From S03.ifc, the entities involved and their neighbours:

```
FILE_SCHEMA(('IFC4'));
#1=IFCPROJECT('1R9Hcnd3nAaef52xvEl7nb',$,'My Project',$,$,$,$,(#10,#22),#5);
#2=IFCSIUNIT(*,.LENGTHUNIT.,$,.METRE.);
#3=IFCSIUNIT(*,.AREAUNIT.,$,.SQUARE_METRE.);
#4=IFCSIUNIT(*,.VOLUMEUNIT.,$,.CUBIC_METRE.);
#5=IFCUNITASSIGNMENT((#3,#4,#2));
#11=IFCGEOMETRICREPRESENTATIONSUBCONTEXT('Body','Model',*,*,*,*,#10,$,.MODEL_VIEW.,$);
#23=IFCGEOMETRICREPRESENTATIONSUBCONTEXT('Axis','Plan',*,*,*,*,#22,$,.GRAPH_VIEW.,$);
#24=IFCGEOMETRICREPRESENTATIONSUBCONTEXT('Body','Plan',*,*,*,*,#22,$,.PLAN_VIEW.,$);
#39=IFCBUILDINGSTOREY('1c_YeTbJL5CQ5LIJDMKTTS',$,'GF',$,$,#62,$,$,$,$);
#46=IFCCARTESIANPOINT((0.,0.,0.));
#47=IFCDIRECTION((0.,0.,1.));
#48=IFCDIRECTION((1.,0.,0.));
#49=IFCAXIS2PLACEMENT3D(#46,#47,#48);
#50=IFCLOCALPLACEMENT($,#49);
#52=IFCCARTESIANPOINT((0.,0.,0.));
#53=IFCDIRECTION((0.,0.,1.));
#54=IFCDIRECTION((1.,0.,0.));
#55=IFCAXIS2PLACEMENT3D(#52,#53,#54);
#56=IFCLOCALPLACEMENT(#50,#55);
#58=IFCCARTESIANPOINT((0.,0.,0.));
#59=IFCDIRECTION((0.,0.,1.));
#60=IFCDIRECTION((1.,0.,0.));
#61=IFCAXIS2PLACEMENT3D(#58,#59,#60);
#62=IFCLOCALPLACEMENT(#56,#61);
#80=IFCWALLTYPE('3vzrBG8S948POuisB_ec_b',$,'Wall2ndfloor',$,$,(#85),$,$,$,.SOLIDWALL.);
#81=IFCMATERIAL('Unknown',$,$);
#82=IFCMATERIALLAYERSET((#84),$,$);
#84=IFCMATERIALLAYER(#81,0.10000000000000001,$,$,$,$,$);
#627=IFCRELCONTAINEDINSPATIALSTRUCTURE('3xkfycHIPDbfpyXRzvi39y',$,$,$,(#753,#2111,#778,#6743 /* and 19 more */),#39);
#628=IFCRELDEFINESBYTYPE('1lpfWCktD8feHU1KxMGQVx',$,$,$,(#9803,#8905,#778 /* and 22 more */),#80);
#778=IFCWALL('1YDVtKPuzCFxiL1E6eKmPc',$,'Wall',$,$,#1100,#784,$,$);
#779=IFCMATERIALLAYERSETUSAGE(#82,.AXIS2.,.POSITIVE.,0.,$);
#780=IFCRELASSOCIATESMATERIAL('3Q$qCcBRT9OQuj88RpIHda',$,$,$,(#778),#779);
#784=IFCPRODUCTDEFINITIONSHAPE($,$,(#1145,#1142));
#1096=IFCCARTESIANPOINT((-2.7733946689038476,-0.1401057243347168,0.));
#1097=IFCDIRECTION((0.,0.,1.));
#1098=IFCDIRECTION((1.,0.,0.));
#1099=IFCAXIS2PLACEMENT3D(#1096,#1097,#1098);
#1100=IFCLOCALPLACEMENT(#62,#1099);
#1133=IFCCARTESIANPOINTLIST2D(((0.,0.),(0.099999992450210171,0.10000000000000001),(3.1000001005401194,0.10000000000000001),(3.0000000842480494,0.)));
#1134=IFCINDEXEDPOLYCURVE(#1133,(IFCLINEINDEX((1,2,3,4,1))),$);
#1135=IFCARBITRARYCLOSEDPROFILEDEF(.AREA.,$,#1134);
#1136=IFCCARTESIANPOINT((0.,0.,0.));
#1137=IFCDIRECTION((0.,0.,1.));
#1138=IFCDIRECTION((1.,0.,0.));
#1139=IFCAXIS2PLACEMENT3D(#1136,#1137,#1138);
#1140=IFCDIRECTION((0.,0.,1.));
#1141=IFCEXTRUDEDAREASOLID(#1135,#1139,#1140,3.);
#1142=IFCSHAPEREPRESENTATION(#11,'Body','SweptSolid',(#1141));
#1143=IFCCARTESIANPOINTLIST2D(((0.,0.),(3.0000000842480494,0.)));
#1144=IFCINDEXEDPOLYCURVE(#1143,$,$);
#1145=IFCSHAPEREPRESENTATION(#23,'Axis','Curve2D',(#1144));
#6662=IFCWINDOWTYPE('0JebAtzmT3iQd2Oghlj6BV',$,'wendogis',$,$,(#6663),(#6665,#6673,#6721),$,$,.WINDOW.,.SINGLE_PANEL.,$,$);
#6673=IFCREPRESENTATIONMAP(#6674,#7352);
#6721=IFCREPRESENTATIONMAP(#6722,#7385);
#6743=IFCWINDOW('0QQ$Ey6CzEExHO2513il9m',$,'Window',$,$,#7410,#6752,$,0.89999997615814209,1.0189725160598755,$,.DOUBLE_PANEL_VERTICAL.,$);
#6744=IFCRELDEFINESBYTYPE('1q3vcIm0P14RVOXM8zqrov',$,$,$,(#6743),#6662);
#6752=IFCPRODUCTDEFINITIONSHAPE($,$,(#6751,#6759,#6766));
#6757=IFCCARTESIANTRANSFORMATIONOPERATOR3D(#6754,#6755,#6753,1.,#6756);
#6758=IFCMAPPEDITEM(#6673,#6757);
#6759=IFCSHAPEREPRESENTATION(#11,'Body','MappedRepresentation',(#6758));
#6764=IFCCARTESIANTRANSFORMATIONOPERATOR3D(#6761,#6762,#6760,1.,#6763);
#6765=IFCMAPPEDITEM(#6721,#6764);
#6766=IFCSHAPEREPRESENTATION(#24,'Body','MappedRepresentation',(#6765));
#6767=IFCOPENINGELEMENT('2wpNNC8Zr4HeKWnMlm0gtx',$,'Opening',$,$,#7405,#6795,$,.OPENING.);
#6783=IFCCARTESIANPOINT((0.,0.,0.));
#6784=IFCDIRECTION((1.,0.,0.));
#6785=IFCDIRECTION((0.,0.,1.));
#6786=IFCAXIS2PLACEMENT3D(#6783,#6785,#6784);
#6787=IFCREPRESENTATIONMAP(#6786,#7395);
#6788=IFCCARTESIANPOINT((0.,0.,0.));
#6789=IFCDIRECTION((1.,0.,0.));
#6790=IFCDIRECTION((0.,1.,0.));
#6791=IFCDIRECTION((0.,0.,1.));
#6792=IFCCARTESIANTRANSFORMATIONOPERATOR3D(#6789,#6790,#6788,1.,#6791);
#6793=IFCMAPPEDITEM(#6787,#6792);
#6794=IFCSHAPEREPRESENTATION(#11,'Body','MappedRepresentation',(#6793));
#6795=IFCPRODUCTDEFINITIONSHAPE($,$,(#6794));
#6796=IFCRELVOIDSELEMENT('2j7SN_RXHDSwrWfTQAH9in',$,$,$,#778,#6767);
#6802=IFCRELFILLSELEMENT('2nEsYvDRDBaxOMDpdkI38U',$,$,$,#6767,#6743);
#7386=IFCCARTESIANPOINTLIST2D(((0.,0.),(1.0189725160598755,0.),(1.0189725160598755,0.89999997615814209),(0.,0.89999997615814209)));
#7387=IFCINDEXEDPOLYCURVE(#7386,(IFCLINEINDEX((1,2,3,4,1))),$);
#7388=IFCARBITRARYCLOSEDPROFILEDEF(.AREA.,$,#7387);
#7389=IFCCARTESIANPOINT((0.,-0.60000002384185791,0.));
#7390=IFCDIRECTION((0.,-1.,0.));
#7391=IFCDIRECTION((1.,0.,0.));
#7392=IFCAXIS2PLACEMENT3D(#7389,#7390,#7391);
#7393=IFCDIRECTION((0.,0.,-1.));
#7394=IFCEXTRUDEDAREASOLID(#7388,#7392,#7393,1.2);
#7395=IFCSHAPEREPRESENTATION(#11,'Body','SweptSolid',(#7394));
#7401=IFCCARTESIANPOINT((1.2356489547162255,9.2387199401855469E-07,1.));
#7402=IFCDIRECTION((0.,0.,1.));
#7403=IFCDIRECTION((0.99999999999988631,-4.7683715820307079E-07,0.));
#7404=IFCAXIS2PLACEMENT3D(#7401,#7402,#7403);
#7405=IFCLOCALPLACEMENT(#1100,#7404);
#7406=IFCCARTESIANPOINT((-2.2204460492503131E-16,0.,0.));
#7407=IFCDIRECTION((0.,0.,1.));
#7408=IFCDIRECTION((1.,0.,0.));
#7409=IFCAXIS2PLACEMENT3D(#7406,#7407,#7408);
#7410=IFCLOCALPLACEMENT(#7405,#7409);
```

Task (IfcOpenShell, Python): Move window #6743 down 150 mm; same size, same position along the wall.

```python
import numpy as np
import ifcopenshell
import ifcopenshell.api.geometry
import ifcopenshell.util.placement
import ifcopenshell.util.unit

model = ifcopenshell.open("S03.ifc")
unit_scale = ifcopenshell.util.unit.calculate_unit_scale(model)

window = model.by_guid("0QQ$Ey6CzEExHO2513il9m")
opening = window.FillsVoids[0].RelatingOpeningElement
dz = -0.15

shift = np.array([0.0, 0.0, dz])
# The window is placed relative to its opening, so it follows when the opening moves.
matrix = ifcopenshell.util.placement.get_local_placement(opening.ObjectPlacement)
matrix[:3, 3] += shift
ifcopenshell.api.geometry.edit_object_placement(
    model, product=opening, matrix=matrix, is_si=False, should_transform_children=True
)

print(f"moved by {dz * unit_scale:+.3f} m")

model.write("S03_updated.ifc")
```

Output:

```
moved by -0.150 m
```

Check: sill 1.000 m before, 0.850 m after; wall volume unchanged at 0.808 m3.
